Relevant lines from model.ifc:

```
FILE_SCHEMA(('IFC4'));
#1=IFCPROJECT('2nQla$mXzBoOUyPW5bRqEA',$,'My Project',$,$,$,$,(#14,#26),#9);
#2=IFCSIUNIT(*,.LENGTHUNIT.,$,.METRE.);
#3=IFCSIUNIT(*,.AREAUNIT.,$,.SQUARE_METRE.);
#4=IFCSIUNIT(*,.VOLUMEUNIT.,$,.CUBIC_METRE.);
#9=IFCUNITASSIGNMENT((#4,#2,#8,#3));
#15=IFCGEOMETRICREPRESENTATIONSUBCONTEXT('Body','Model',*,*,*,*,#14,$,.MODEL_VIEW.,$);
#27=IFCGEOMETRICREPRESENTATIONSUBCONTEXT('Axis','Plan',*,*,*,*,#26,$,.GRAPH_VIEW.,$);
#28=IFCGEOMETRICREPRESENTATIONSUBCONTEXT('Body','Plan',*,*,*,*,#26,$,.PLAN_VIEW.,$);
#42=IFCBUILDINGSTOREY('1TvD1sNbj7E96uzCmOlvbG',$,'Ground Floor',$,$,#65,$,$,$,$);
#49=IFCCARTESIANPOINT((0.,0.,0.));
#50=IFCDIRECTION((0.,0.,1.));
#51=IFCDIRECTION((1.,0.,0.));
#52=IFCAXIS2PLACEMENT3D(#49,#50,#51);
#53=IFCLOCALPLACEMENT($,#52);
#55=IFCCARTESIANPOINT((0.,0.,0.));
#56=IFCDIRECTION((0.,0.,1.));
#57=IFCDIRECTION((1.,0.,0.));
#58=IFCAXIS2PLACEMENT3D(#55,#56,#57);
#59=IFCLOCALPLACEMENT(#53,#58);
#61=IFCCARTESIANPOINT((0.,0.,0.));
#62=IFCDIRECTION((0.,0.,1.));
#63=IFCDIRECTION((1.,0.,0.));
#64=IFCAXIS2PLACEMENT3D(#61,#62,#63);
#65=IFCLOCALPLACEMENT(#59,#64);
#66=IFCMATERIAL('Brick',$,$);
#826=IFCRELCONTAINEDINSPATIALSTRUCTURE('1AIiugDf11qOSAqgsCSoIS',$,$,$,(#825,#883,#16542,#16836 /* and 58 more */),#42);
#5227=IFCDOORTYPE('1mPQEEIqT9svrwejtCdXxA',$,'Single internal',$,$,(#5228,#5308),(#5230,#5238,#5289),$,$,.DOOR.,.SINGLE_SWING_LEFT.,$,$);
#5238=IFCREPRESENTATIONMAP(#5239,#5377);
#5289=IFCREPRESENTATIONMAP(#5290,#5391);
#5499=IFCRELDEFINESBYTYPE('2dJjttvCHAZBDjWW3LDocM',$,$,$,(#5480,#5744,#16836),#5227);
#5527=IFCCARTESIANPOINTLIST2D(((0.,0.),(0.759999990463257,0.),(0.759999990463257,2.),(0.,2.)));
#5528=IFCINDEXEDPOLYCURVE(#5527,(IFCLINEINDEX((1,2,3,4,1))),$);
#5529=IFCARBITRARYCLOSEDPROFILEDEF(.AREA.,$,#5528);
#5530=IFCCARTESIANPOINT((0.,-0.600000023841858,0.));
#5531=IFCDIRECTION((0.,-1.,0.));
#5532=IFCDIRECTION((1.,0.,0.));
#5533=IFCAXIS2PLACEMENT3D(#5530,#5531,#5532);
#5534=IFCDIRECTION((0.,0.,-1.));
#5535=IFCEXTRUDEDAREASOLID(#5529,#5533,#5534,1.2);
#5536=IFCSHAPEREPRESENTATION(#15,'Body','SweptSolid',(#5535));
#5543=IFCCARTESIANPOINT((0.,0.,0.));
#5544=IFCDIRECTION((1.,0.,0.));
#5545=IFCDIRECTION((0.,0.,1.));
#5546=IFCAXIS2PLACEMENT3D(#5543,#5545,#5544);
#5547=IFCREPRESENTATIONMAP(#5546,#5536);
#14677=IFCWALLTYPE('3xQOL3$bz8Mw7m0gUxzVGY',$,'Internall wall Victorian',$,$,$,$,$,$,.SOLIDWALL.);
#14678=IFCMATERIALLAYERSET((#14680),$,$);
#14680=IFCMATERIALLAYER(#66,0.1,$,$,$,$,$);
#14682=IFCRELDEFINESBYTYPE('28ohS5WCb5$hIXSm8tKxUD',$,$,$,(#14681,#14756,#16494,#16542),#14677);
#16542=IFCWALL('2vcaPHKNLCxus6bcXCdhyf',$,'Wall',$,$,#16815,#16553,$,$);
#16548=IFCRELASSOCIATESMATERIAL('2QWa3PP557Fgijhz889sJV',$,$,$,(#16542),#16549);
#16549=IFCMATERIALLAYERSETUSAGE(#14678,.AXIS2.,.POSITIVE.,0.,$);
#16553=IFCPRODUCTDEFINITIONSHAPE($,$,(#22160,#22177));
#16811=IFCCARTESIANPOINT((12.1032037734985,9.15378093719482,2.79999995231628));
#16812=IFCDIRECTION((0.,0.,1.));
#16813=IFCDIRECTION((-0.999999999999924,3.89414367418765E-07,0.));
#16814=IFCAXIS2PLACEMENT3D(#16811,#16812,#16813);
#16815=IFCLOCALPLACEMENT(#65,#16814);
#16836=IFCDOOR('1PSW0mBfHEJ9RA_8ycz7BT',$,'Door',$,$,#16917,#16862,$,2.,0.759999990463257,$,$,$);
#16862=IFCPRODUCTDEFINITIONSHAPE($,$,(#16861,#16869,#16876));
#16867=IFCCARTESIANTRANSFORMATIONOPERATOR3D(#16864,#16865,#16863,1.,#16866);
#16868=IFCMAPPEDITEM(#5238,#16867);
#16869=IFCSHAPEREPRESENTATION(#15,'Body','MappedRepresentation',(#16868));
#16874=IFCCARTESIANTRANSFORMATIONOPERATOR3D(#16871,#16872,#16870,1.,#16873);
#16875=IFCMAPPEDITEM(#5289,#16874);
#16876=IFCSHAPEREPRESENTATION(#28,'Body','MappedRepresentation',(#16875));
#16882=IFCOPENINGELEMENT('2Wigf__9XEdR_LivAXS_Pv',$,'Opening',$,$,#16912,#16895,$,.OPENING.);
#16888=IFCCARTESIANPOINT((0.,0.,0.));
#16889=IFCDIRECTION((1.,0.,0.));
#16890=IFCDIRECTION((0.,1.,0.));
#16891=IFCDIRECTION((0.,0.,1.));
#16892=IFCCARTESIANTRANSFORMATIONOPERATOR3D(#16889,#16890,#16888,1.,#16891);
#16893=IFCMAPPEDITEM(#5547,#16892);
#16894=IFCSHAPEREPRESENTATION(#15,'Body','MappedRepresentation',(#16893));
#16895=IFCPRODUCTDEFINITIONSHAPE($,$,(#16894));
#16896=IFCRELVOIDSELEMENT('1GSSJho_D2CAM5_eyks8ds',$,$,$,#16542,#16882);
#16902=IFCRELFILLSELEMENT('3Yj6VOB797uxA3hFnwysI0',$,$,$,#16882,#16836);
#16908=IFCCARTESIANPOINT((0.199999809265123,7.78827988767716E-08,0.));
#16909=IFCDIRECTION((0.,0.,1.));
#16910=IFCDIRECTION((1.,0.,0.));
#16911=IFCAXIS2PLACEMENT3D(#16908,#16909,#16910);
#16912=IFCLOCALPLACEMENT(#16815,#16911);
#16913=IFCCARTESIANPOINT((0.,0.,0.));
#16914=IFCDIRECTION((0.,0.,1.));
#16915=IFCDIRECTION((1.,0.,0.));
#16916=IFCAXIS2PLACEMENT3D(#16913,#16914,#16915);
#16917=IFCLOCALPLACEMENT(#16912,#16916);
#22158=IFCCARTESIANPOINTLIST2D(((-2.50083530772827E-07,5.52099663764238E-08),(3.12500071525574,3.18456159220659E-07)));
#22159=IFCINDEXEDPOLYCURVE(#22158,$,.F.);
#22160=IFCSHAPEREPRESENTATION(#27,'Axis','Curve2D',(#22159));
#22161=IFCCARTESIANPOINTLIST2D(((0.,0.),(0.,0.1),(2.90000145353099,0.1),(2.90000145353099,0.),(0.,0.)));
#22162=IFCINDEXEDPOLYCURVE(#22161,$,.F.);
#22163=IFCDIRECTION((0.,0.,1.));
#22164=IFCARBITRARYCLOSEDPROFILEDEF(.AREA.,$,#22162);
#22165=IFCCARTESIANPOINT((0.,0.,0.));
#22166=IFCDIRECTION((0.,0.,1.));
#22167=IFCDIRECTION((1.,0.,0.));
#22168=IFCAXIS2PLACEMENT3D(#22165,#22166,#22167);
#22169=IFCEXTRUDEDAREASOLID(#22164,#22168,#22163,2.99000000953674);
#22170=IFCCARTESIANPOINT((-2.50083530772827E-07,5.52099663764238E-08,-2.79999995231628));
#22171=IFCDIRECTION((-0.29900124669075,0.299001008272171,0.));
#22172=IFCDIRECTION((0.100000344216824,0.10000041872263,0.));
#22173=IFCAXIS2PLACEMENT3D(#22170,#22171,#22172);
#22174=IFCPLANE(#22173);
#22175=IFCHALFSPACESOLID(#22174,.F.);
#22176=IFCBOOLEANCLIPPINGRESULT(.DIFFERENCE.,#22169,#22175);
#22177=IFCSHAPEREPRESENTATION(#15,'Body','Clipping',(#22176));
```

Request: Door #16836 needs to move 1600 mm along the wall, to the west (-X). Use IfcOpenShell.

```python
import ifcopenshell
import ifcopenshell.api.geometry
import ifcopenshell.util.placement
import ifcopenshell.util.unit

model = ifcopenshell.open("model.ifc")
unit_scale = ifcopenshell.util.unit.calculate_unit_scale(model)

door = model.by_guid("1PSW0mBfHEJ9RA_8ycz7BT")
opening = door.FillsVoids[0].RelatingOpeningElement
wall = opening.VoidsElements[0].RelatingBuildingElement

wall_matrix = ifcopenshell.util.placement.get_local_placement(wall.ObjectPlacement)
shift = wall_matrix[:3, 0] * 1.6 / unit_scale
before = ifcopenshell.util.placement.get_local_placement(door.ObjectPlacement)[:3, 3].copy()

# The door is placed relative to its opening, so it follows when the opening moves.
matrix = ifcopenshell.util.placement.get_local_placement(opening.ObjectPlacement)
matrix[:3, 3] += shift
ifcopenshell.api.geometry.edit_object_placement(
    model, product=opening, matrix=matrix, is_si=False, should_transform_children=True
)

after = ifcopenshell.util.placement.get_local_placement(door.ObjectPlacement)[:3, 3]
print("door moved by", (after - before).round(3) + 0.0)

model.write("model_v2.ifc")
```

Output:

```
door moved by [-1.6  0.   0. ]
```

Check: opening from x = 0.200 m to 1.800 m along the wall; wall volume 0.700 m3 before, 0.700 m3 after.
